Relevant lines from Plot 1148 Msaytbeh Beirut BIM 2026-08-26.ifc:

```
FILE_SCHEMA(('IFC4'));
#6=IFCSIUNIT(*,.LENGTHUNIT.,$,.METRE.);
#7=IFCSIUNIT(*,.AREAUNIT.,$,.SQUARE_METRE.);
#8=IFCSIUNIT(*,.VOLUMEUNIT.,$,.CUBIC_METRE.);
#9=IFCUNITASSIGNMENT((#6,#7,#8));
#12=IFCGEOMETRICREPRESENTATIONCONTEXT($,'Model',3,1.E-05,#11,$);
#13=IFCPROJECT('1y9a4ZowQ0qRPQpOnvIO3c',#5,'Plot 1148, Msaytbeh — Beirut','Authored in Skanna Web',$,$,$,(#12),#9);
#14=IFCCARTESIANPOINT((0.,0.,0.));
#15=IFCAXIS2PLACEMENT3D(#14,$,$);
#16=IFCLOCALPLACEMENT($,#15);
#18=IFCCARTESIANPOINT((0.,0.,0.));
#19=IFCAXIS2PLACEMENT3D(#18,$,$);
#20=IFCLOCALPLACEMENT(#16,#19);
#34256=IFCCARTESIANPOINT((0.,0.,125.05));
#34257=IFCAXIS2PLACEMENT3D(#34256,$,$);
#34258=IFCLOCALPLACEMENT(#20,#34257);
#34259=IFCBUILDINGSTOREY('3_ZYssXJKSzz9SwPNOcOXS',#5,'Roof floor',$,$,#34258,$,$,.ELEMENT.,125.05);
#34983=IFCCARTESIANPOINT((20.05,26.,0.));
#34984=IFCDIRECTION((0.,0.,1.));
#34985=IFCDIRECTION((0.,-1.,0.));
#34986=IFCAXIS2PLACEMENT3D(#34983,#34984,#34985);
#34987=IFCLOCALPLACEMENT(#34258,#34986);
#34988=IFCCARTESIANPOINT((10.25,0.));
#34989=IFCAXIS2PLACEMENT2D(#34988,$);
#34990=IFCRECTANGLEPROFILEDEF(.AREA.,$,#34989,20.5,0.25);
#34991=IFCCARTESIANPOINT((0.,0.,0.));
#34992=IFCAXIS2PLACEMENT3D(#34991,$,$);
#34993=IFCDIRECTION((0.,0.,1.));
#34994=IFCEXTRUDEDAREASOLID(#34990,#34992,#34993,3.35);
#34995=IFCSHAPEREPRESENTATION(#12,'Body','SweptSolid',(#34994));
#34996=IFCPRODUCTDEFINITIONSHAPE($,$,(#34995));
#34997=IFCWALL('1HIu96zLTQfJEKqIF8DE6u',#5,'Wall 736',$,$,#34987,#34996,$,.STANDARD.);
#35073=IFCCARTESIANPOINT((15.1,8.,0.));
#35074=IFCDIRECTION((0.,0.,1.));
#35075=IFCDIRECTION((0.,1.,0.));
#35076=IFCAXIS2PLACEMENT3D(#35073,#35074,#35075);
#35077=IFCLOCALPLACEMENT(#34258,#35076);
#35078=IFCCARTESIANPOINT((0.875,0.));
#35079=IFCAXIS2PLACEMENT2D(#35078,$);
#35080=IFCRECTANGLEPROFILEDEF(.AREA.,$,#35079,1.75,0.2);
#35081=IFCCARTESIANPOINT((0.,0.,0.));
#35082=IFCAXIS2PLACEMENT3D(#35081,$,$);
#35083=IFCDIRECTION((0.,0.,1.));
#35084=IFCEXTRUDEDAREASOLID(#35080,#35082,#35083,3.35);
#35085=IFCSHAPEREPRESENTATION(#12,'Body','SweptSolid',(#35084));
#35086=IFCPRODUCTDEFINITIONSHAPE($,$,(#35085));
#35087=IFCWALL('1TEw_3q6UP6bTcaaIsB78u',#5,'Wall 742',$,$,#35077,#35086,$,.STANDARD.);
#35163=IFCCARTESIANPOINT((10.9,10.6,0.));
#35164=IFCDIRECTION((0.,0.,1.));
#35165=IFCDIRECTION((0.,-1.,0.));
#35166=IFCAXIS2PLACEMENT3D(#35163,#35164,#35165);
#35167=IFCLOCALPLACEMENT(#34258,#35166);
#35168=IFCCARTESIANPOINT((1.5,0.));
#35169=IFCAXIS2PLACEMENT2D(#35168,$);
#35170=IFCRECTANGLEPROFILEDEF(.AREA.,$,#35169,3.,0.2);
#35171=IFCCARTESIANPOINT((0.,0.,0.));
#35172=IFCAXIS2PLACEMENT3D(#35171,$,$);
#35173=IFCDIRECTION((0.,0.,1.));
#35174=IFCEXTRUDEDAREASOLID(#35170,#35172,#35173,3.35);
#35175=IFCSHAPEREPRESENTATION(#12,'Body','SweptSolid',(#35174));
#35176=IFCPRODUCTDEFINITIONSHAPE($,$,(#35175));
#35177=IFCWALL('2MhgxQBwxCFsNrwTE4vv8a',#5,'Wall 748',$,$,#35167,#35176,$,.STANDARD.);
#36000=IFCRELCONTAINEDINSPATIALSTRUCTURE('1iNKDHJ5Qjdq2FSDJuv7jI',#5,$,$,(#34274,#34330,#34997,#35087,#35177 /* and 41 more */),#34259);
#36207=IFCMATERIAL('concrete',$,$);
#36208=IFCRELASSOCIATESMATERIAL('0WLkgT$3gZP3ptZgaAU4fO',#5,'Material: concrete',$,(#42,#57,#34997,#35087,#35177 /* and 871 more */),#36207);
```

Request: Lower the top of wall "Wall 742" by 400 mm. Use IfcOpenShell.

```python
import ifcopenshell
import ifcopenshell.geom
import ifcopenshell.util.shape
import ifcopenshell.util.unit

model = ifcopenshell.open("Plot 1148 Msaytbeh Beirut BIM 2026-08-26.ifc")
unit_scale = ifcopenshell.util.unit.calculate_unit_scale(model)
settings = ifcopenshell.geom.settings()


def volume(element):
    """Net volume in cubic metres, openings subtracted."""
    shape = ifcopenshell.geom.create_shape(settings, element)
    return ifcopenshell.util.shape.get_volume(shape.geometry)


wall = model.by_guid("1TEw_3q6UP6bTcaaIsB78u")
before = volume(wall)

body = next(r for r in wall.Representation.Representations if r.RepresentationIdentifier == "Body")
solid = body.Items[0]
old_height = solid.Depth
solid.Depth -= 0.4 / unit_scale
after = volume(wall)

print(f"height {old_height:g} -> {solid.Depth:g}, volume {before:.3f} -> {after:.3f} m3")

model.write("Plot 1148 Msaytbeh Beirut BIM 2026-08-26_rev.ifc")
```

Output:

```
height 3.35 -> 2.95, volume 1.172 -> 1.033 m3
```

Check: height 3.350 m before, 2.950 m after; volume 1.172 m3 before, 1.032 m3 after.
